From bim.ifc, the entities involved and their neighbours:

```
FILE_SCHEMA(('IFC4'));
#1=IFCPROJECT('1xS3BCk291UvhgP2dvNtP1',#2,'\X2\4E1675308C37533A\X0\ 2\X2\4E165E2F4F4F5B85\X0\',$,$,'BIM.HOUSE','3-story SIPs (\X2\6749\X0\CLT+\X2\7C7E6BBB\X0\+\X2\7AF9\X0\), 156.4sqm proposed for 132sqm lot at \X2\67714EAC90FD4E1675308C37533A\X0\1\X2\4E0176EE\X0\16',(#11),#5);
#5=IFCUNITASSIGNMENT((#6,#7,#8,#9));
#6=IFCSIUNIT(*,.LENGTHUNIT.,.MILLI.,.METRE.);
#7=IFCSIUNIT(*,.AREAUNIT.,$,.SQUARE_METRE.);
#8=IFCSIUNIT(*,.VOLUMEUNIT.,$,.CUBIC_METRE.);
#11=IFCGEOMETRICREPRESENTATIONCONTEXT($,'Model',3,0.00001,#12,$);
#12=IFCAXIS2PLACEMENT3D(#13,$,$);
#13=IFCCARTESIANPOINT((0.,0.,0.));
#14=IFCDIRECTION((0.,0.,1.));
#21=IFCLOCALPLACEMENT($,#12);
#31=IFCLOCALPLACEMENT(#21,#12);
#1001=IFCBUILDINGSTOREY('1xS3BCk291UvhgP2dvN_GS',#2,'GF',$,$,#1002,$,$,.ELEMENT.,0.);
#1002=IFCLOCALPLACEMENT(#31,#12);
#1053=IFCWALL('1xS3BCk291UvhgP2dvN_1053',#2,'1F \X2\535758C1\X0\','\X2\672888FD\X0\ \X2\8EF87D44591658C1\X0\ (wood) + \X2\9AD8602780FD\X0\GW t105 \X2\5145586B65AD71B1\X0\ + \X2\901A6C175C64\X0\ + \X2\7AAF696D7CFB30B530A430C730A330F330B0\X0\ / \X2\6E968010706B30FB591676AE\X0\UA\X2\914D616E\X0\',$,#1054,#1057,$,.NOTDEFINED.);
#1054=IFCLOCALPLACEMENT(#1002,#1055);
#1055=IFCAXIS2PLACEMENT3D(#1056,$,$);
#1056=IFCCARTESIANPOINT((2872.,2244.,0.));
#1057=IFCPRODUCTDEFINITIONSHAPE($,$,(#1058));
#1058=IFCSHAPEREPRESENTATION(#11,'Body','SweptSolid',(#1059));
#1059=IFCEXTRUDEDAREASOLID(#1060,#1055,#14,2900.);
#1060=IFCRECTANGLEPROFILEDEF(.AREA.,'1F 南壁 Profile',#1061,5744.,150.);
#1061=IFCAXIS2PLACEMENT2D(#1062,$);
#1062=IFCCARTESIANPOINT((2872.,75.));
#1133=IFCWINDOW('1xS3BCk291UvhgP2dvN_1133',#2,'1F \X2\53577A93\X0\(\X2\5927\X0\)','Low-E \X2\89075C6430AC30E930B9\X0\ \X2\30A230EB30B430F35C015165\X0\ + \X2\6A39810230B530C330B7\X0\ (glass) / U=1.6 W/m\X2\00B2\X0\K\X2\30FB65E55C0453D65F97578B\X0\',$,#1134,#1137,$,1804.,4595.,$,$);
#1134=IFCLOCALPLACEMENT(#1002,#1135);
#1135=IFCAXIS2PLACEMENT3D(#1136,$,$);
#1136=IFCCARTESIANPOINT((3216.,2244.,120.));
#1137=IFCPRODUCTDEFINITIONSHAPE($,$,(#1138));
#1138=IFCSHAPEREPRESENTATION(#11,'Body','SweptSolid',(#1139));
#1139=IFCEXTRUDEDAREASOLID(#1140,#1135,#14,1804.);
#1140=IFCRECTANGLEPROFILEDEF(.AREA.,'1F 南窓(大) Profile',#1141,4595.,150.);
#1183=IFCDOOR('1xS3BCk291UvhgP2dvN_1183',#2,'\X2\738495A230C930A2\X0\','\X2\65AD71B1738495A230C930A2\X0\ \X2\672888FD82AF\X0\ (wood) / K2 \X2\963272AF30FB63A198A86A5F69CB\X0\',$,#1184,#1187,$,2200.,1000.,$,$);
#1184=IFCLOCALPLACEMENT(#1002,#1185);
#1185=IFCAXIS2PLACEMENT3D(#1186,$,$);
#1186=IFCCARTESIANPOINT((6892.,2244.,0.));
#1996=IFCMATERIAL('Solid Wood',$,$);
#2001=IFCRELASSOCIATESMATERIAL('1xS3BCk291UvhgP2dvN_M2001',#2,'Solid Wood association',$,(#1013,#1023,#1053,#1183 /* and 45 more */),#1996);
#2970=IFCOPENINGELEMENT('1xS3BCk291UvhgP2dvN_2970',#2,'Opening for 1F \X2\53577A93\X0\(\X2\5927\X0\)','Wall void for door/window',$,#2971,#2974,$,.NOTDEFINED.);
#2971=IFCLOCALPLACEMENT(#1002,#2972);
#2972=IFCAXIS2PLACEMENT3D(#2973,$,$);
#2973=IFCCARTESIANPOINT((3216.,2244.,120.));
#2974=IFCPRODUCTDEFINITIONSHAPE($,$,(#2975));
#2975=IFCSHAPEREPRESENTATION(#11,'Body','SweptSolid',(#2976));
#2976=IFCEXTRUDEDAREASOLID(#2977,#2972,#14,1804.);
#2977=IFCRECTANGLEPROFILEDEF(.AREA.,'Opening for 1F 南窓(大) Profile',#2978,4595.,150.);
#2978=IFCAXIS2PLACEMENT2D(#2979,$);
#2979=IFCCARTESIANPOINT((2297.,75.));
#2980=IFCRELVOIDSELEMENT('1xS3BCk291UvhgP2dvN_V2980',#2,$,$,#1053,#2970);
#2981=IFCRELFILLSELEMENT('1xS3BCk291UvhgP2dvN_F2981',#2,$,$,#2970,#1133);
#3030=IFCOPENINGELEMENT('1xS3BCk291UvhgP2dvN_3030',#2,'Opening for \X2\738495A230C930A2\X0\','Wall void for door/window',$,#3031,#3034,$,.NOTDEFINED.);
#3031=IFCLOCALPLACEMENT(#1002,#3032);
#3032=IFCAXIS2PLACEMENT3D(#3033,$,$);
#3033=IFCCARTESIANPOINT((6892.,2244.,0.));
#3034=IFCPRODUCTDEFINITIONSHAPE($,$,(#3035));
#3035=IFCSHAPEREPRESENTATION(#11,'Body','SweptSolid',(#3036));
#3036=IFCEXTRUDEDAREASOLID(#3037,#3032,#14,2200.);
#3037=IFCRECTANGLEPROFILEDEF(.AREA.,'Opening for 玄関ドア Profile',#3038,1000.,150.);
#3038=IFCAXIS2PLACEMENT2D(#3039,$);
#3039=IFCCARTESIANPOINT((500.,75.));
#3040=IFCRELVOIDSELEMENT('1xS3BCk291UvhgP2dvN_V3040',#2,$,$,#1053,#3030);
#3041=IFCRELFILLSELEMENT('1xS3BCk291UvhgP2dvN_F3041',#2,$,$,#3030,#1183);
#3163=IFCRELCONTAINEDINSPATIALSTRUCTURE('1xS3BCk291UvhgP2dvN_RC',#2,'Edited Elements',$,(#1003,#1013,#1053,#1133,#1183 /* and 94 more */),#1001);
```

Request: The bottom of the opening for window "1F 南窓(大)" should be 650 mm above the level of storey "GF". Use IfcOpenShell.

```python
import numpy as np
import ifcopenshell
import ifcopenshell.api.geometry
import ifcopenshell.geom
import ifcopenshell.util.element
import ifcopenshell.util.placement
import ifcopenshell.util.shape
import ifcopenshell.util.unit

model = ifcopenshell.open("bim.ifc")
unit_scale = ifcopenshell.util.unit.calculate_unit_scale(model)

window = model.by_guid("1xS3BCk291UvhgP2dvN_1133")
opening = window.FillsVoids[0].RelatingOpeningElement
storey = ifcopenshell.util.element.get_container(window, ifc_class="IfcBuildingStorey")
level = ifcopenshell.util.placement.get_local_placement(storey.ObjectPlacement)[2, 3]

# The opening's origin need not be at the sill, so measure its lowest point.
shape = ifcopenshell.geom.create_shape(ifcopenshell.geom.settings(), opening)
bottom = ifcopenshell.util.shape.get_shape_bottom_elevation(shape, shape.geometry) / unit_scale
dz = level + 650.0 - bottom

shift = np.array([0.0, 0.0, dz])
# The window is not placed relative to its opening, so move both.
for product in (opening, window):
    matrix = ifcopenshell.util.placement.get_local_placement(product.ObjectPlacement)
    matrix[:3, 3] += shift
    ifcopenshell.api.geometry.edit_object_placement(model, product=product, matrix=matrix, is_si=False)

print(f"moved by {dz * unit_scale:+.3f} m")

model.write("bim_updated.ifc")
```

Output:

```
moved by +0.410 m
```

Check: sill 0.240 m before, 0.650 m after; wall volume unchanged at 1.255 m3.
